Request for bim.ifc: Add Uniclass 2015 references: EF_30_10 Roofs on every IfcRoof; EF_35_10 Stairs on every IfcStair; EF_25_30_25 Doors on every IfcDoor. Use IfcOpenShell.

First a look at what the model holds.

```python
import ifcopenshell

model = ifcopenshell.open("bim.ifc")
print(model.schema)
print("classifications:", [c.Name for c in model.by_type("IfcClassification")])
for ifc_class in ("IfcDoor", "IfcRoof", "IfcStair", "IfcWall", "IfcWindow"):
    print(ifc_class, len(model.by_type(ifc_class)))
```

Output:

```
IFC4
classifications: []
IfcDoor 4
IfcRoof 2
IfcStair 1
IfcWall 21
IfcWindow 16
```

```python
import ifcopenshell
import ifcopenshell.api.classification

model = ifcopenshell.open("bim.ifc")

system = ifcopenshell.api.classification.add_classification(model, classification="Uniclass 2015")

codes = {
    "IfcRoof": ("EF_30_10", "Roofs"),
    "IfcStair": ("EF_35_10", "Stairs"),
    "IfcDoor": ("EF_25_30_25", "Doors"),
}
for ifc_class, (code, name) in codes.items():
    products = model.by_type(ifc_class)
    ifcopenshell.api.classification.add_reference(
        model, products=products, classification=system, identification=code, name=name
    )
    print(code, len(products))

model.write("bim_rev.ifc")
```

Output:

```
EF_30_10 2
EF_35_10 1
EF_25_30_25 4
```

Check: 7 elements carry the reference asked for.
